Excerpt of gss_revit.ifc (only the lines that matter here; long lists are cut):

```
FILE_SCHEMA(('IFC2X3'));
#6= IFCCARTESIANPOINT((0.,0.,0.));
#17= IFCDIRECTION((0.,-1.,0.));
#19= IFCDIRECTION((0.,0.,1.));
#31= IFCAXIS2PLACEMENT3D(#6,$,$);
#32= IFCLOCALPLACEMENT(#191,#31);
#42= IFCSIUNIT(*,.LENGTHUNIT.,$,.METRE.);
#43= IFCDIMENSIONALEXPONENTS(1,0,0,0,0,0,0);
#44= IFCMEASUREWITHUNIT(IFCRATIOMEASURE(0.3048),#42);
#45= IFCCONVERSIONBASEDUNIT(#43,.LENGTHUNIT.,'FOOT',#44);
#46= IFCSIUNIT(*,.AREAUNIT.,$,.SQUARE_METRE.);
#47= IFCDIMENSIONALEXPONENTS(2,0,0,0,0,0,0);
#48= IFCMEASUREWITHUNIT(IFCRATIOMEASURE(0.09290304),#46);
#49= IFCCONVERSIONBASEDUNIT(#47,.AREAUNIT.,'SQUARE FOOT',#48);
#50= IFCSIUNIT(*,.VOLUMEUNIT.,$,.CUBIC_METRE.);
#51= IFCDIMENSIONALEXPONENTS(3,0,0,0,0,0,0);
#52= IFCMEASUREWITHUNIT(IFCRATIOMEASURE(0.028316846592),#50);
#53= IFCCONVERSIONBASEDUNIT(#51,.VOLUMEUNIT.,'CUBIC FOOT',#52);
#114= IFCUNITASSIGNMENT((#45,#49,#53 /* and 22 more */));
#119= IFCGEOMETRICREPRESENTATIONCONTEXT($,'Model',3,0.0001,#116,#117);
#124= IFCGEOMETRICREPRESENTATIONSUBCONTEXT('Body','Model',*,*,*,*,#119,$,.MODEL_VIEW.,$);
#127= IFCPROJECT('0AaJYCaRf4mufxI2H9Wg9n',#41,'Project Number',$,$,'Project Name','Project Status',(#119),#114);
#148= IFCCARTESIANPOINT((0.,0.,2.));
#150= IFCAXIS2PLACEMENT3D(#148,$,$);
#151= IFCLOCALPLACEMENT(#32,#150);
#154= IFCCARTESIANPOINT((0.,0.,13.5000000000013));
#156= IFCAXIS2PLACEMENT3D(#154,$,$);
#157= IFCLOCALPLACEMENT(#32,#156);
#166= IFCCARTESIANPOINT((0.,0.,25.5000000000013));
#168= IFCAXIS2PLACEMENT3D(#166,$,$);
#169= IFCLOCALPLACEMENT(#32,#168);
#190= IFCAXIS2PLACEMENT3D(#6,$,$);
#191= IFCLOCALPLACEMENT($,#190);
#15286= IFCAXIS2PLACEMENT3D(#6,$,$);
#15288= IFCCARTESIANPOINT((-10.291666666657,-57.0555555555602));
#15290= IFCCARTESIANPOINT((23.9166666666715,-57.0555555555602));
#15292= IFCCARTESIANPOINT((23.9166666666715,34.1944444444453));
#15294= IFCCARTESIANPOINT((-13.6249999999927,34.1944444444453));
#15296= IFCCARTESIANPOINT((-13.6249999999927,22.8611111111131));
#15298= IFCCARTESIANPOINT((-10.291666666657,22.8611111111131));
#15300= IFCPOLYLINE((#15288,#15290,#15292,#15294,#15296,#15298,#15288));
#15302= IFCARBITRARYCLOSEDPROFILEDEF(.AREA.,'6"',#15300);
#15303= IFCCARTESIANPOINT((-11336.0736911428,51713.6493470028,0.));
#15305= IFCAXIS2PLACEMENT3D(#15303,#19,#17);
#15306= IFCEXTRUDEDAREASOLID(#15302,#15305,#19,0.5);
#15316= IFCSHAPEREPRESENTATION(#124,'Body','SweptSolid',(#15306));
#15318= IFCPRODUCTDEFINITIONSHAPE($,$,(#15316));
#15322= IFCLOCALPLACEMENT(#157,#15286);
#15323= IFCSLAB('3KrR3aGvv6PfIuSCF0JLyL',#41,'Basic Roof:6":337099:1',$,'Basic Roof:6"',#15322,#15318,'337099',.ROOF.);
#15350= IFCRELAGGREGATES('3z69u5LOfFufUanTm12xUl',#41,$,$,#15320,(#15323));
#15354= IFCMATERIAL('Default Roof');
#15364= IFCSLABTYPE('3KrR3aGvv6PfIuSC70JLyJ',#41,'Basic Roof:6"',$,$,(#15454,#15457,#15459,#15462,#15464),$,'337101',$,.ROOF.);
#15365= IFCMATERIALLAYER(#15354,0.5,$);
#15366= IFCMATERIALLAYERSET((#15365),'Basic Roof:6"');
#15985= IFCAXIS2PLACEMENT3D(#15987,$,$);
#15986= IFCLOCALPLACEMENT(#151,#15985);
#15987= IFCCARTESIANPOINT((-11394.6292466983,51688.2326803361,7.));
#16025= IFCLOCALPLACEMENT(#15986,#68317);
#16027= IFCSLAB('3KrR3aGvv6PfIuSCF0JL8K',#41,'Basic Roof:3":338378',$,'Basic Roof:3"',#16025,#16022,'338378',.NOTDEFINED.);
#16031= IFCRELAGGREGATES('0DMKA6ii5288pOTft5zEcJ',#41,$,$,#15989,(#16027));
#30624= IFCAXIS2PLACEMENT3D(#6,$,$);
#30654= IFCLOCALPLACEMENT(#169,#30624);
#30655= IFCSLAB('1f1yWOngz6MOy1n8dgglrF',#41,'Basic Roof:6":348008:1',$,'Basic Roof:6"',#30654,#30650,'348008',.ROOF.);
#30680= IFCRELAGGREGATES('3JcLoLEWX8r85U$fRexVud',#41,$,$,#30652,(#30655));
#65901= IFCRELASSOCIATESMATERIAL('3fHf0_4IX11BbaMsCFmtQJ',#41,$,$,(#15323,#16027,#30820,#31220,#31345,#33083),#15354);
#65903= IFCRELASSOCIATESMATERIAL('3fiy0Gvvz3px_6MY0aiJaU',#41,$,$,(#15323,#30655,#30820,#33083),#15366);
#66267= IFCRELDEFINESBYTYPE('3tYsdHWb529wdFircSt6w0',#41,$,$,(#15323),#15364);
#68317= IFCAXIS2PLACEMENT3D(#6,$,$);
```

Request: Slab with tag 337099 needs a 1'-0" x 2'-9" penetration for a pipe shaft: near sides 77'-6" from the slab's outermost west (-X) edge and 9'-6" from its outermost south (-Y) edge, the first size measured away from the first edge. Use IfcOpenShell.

```python
import numpy as np
import ifcopenshell
import ifcopenshell.api.feature
import ifcopenshell.api.geometry
import ifcopenshell.api.root
import ifcopenshell.geom
import ifcopenshell.util.placement
import ifcopenshell.util.representation
import ifcopenshell.util.shape
import ifcopenshell.util.unit

model = ifcopenshell.open("gss_revit.ifc")
unit_scale = ifcopenshell.util.unit.calculate_unit_scale(model)
settings = ifcopenshell.geom.settings()


def volume(element):
    """Net volume in cubic metres, openings subtracted."""
    shape = ifcopenshell.geom.create_shape(settings, element)
    return ifcopenshell.util.shape.get_volume(shape.geometry)


slab = model.by_guid("3KrR3aGvv6PfIuSCF0JLyL")
before = volume(slab)

# Extent in the slab's own axes, in metres. The edges named are its -X and -Y sides.
slab_shape = ifcopenshell.geom.create_shape(settings, slab)
vertices = ifcopenshell.util.shape.get_vertices(slab_shape.geometry)
x_min, y_min, bottom = vertices.min(axis=0)
top = vertices[:, 2].max()

opening = ifcopenshell.api.root.create_entity(model, ifc_class="IfcOpeningElement", name="Pipe shaft opening")
context = ifcopenshell.util.representation.get_context(model, "Model", "Body", "MODEL_VIEW")
width, depth = 0.3048, 0.8382
outline = [(0.0, 0.0), (width, 0.0), (width, depth), (0.0, depth), (0.0, 0.0)]
# Overshoot both faces by 50 mm so the cut is clean.
shape = ifcopenshell.api.geometry.add_slab_representation(
    model, context=context, depth=top - bottom + 0.1, polyline=outline
)
ifcopenshell.api.geometry.assign_representation(model, product=opening, representation=shape)

matrix = ifcopenshell.util.placement.get_local_placement(slab.ObjectPlacement)
matrix[:, 3] = matrix @ np.append(np.array([x_min + 23.622, y_min + 2.8956, bottom - 0.05]) / unit_scale, 1.0)
ifcopenshell.api.geometry.edit_object_placement(model, product=opening, matrix=matrix, is_si=False)
ifcopenshell.api.feature.add_feature(model, feature=opening, element=slab)

after = volume(slab)

print(f"slab volume {before:.3f} -> {after:.3f} m3")

model.write("gss_revit_v2.ifc")
```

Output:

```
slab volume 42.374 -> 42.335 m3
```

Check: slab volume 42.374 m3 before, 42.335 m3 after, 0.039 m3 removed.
